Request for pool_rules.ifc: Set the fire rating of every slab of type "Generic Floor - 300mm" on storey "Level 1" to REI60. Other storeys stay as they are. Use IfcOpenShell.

First a look at what the model holds.

```python
import ifcopenshell
import ifcopenshell.util.element

model = ifcopenshell.open("pool_rules.ifc")
print(model.schema)
storey = next(s for s in model.by_type("IfcBuildingStorey") if s.Name == "Level 1")
slabs = [e for e in ifcopenshell.util.element.get_decomposition(storey) if e.is_a("IfcSlab")]
seen = {}
for e in slabs:
    element_type = ifcopenshell.util.element.get_type(e)
    key = (element_type.Name if element_type != e and element_type else None, ifcopenshell.util.element.get_pset(e, "Pset_SlabCommon", "FireRating"))
    seen[key] = seen.get(key, 0) + 1
for (name, value), count in sorted(seen.items(), key=str):
    print(count, "x", name, "|", value)
```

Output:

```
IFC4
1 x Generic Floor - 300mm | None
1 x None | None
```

```python
import ifcopenshell
import ifcopenshell.api.pset
import ifcopenshell.util.element

model = ifcopenshell.open("pool_rules.ifc")

storey = next(s for s in model.by_type("IfcBuildingStorey") if s.Name == "Level 1")
slabs = [e for e in ifcopenshell.util.element.get_decomposition(storey) if e.is_a("IfcSlab")]

count = 0
for e in slabs:
    element_type = ifcopenshell.util.element.get_type(e)
    if element_type in (None, e) or element_type.Name != "Generic Floor - 300mm":
        continue
    # add_pset returns the element's existing set when there is one.
    pset = ifcopenshell.api.pset.add_pset(model, product=e, name="Pset_SlabCommon")
    ifcopenshell.api.pset.edit_pset(model, pset=pset, properties={"FireRating": "REI60"})
    count += 1

print(count, "slabs updated")

model.write("pool_rules_rev.ifc")
```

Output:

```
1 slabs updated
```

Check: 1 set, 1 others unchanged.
